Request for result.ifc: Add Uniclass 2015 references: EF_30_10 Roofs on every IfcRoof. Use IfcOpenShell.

First a look at what the model holds.

```python
import ifcopenshell

model = ifcopenshell.open("result.ifc")
print(model.schema)
print("classifications:", [c.Name for c in model.by_type("IfcClassification")])
for ifc_class in ("IfcDoor", "IfcRoof", "IfcStair", "IfcWall", "IfcWindow"):
    print(ifc_class, len(model.by_type(ifc_class)))
```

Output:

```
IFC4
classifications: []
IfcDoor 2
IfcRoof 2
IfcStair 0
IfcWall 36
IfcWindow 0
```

```python
import ifcopenshell
import ifcopenshell.api.classification

model = ifcopenshell.open("result.ifc")

system = ifcopenshell.api.classification.add_classification(model, classification="Uniclass 2015")

codes = {
    "IfcRoof": ("EF_30_10", "Roofs"),
}
for ifc_class, (code, name) in codes.items():
    products = model.by_type(ifc_class)
    ifcopenshell.api.classification.add_reference(
        model, products=products, classification=system, identification=code, name=name
    )
    print(code, len(products))

model.write("result_updated.ifc")
```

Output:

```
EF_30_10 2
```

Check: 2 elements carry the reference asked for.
